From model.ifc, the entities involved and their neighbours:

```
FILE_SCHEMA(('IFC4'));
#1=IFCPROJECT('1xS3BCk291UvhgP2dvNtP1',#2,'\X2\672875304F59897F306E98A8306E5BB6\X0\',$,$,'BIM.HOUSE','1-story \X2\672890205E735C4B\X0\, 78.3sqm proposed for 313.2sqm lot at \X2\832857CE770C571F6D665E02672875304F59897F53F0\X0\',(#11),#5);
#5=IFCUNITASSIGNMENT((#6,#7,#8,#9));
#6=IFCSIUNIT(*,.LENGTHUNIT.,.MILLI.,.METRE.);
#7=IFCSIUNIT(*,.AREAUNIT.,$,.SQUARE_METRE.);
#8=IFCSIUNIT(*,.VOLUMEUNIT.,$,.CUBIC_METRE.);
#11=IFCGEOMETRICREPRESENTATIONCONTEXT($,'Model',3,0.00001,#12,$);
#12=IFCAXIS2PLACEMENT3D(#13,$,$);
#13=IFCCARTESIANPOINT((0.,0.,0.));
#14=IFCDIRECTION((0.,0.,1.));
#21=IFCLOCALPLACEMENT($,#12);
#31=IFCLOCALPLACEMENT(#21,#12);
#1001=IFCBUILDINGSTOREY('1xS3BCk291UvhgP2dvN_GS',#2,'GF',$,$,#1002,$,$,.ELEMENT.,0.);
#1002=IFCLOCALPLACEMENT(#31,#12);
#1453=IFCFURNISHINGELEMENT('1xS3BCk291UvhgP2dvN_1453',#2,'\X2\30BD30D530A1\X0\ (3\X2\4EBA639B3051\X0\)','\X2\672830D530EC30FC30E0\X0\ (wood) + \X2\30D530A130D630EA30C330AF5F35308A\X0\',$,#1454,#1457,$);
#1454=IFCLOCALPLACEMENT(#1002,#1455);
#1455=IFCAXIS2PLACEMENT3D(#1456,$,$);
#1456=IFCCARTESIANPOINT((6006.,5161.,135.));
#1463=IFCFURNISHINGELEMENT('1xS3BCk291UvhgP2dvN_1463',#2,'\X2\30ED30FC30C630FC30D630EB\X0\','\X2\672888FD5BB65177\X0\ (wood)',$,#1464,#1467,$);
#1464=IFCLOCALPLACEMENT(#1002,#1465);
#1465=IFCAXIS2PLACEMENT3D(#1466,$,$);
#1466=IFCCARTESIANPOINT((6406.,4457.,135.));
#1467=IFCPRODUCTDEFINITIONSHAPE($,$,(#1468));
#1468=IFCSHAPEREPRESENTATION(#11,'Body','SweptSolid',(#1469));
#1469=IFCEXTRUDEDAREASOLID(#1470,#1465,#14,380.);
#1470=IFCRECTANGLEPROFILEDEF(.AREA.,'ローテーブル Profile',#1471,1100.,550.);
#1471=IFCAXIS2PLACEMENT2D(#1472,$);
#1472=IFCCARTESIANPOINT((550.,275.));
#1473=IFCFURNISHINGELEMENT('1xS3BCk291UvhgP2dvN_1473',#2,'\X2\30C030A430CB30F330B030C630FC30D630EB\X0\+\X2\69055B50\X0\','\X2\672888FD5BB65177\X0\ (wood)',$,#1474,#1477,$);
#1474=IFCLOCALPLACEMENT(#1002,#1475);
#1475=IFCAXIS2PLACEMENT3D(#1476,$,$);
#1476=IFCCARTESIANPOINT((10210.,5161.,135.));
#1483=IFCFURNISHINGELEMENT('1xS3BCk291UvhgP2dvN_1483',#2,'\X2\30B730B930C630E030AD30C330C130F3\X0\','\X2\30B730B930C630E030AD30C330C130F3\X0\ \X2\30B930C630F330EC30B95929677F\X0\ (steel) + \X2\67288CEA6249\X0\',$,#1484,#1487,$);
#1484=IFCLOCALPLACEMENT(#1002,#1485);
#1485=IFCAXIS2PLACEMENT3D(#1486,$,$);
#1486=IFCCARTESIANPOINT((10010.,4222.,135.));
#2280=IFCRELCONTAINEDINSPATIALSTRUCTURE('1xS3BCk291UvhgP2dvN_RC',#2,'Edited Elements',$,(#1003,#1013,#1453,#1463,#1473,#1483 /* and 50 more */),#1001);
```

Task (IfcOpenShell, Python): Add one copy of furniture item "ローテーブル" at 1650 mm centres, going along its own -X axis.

```python
import ifcopenshell
import ifcopenshell.api.geometry
import ifcopenshell.api.root
import ifcopenshell.util.element
import ifcopenshell.util.placement
import ifcopenshell.util.unit

model = ifcopenshell.open("model.ifc")
unit_scale = ifcopenshell.util.unit.calculate_unit_scale(model)


def reuse_history(source, copy):
    """copy_class also copies each property set's owner history, people and application; keep the originals."""
    for rel in copy.IsDefinedBy:
        if rel.is_a("IfcRelDefinesByProperties") and (history := rel.RelatingPropertyDefinition.OwnerHistory):
            rel.RelatingPropertyDefinition.OwnerHistory = source.OwnerHistory
            ifcopenshell.util.element.remove_deep2(model, history)


source = model.by_id(1463)
base = ifcopenshell.util.placement.get_local_placement(source.ObjectPlacement)
step = -base[:3, 0] * 1.65 / unit_scale

for i in range(1, 2):
    copy = ifcopenshell.api.root.copy_class(model, product=source)
    copy.Representation = ifcopenshell.util.element.copy_deep(
        model, source.Representation, exclude=["IfcGeometricRepresentationContext", "IfcRepresentationMap"]
    )
    reuse_history(source, copy)
    matrix = base.copy()
    matrix[:3, 3] += i * step
    print("added at", matrix[:3, 3].round(3) + 0.0)
    ifcopenshell.api.geometry.edit_object_placement(model, product=copy, matrix=matrix, is_si=False)

model.write("model-out.ifc")
```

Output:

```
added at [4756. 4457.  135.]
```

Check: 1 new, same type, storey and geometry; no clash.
